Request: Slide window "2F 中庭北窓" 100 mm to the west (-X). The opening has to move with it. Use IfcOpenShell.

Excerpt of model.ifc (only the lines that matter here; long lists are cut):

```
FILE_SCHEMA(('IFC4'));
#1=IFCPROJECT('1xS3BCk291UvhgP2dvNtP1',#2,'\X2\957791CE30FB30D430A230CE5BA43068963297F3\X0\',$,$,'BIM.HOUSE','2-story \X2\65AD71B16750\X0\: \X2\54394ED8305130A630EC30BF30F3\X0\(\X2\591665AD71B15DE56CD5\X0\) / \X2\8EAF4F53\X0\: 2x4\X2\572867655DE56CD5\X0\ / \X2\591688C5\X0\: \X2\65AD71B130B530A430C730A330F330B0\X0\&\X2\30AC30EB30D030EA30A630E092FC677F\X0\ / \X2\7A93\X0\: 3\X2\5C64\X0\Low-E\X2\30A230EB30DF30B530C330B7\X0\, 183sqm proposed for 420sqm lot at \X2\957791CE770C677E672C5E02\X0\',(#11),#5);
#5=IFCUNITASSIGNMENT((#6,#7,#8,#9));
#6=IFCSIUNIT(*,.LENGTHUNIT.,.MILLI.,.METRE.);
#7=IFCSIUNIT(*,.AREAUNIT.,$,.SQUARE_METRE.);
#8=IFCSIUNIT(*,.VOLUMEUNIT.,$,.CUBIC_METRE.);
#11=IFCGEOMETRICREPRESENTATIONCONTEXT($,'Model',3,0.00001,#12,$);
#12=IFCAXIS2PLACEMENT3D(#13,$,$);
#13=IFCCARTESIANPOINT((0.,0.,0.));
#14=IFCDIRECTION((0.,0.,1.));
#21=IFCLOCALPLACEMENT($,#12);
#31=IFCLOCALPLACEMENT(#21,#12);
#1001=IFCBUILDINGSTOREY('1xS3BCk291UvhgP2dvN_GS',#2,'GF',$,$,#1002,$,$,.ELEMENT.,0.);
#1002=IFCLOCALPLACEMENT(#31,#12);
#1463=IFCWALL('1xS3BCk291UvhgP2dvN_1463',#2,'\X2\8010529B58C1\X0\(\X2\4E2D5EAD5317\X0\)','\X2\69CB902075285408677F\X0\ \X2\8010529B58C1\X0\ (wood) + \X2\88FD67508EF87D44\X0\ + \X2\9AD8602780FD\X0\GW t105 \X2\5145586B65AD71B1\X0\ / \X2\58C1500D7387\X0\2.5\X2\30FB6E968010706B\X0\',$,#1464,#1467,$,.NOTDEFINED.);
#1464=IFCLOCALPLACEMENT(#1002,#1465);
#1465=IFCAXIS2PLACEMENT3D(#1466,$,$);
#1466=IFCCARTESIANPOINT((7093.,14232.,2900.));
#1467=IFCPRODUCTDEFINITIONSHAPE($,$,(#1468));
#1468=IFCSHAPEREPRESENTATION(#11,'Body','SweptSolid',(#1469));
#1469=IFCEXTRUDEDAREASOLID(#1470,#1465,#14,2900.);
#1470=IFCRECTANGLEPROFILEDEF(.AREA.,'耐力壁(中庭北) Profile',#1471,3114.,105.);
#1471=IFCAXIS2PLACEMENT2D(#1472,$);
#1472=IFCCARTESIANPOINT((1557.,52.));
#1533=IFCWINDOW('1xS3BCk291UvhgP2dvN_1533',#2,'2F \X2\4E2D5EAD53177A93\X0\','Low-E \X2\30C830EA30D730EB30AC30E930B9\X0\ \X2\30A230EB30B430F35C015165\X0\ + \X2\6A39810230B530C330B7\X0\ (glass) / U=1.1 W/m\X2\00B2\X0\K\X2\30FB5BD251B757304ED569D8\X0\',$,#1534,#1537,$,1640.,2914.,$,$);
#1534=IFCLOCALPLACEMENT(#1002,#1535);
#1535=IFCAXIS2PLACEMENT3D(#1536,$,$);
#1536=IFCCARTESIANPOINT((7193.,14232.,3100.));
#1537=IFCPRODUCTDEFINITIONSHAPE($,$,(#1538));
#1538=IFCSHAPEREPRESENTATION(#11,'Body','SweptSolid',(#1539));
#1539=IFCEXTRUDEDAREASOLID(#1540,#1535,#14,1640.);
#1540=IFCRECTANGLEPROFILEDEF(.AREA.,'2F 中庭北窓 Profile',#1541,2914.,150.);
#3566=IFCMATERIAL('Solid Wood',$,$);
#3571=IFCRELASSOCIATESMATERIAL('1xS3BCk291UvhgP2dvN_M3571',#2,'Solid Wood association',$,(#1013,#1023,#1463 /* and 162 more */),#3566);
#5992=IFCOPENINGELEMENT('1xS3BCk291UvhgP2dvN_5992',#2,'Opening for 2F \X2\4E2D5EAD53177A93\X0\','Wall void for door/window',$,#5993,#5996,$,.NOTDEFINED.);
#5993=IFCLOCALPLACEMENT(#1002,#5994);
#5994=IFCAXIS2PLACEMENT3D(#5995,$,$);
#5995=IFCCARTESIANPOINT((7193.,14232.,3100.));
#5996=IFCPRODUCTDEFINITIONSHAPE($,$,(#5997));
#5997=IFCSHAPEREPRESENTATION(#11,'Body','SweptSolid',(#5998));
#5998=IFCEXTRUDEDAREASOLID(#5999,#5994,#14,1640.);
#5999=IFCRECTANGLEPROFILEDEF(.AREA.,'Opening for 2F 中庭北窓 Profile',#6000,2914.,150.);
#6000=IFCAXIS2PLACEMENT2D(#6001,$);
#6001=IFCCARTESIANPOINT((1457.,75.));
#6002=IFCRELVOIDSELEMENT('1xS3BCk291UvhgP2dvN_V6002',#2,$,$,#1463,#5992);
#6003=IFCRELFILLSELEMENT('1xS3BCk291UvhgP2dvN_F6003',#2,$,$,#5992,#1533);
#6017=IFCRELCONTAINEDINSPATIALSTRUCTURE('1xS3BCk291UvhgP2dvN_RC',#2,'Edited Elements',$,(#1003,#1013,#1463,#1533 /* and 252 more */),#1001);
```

```python
import ifcopenshell
import ifcopenshell.api.geometry
import ifcopenshell.util.placement

model = ifcopenshell.open("model.ifc")

window = model.by_guid("1xS3BCk291UvhgP2dvN_1533")
opening = window.FillsVoids[0].RelatingOpeningElement
wall = opening.VoidsElements[0].RelatingBuildingElement

wall_matrix = ifcopenshell.util.placement.get_local_placement(wall.ObjectPlacement)
shift = wall_matrix[:3, 0] * -100.0
before = ifcopenshell.util.placement.get_local_placement(window.ObjectPlacement)[:3, 3].copy()

# The window is not placed relative to its opening, so move both.
for product in (opening, window):
    matrix = ifcopenshell.util.placement.get_local_placement(product.ObjectPlacement)
    matrix[:3, 3] += shift
    ifcopenshell.api.geometry.edit_object_placement(model, product=product, matrix=matrix, is_si=False)

after = ifcopenshell.util.placement.get_local_placement(window.ObjectPlacement)[:3, 3]
print("window moved by", (after - before).round(3) + 0.0)

model.write("model_updated.ifc")
```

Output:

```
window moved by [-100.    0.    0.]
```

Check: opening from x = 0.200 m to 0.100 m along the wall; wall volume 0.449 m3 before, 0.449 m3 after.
